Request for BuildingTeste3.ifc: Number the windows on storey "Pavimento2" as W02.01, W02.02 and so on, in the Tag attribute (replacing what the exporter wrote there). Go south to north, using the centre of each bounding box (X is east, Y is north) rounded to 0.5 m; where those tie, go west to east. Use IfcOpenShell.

First a look at what the model holds.

```python
import ifcopenshell
import ifcopenshell.util.element
import ifcopenshell.util.placement

model = ifcopenshell.open("BuildingTeste3.ifc")
print(model.schema)
storey = next(s for s in model.by_type("IfcBuildingStorey") if s.Name == "Pavimento2")
windows = [e for e in ifcopenshell.util.element.get_decomposition(storey) if e.is_a("IfcWindow")]
for e in sorted(windows, key=lambda e: e.id()):
    origin = ifcopenshell.util.placement.get_local_placement(e.ObjectPlacement)[:3, 3]
    print(e.id(), e.Tag, e.Name, origin.round(2) + 0.0, sep=" | ")
```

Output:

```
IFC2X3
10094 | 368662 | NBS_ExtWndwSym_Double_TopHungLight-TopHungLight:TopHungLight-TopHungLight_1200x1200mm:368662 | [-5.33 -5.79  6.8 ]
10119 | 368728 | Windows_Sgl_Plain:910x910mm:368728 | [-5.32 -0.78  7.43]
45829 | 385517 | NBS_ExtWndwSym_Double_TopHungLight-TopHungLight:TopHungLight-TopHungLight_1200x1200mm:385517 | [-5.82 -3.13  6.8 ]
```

```python
import ifcopenshell
import ifcopenshell.geom
import ifcopenshell.util.element
import ifcopenshell.util.shape

model = ifcopenshell.open("BuildingTeste3.ifc")
settings = ifcopenshell.geom.settings()
settings.set("use-world-coords", True)


def centre(element):
    shape = ifcopenshell.geom.create_shape(settings, element)
    return ifcopenshell.util.shape.get_bbox_centroid(shape.geometry)


storey = next(s for s in model.by_type("IfcBuildingStorey") if s.Name == "Pavimento2")
windows = [e for e in ifcopenshell.util.element.get_decomposition(storey) if e.is_a("IfcWindow")]

# Insertion points can sit at a corner or the storey origin, so sort by the geometry (in metres).
centres = {e: centre(e) for e in windows}
windows.sort(key=lambda e: (round(centres[e][1] / 0.5), centres[e][0]))

for i, e in enumerate(windows, start=1):
    number = f"W02.{i:02d}"
    e.Tag = number
    print(e.id(), number)

model.write("BuildingTeste3_v2.ifc")
```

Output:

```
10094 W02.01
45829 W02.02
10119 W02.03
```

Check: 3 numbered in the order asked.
